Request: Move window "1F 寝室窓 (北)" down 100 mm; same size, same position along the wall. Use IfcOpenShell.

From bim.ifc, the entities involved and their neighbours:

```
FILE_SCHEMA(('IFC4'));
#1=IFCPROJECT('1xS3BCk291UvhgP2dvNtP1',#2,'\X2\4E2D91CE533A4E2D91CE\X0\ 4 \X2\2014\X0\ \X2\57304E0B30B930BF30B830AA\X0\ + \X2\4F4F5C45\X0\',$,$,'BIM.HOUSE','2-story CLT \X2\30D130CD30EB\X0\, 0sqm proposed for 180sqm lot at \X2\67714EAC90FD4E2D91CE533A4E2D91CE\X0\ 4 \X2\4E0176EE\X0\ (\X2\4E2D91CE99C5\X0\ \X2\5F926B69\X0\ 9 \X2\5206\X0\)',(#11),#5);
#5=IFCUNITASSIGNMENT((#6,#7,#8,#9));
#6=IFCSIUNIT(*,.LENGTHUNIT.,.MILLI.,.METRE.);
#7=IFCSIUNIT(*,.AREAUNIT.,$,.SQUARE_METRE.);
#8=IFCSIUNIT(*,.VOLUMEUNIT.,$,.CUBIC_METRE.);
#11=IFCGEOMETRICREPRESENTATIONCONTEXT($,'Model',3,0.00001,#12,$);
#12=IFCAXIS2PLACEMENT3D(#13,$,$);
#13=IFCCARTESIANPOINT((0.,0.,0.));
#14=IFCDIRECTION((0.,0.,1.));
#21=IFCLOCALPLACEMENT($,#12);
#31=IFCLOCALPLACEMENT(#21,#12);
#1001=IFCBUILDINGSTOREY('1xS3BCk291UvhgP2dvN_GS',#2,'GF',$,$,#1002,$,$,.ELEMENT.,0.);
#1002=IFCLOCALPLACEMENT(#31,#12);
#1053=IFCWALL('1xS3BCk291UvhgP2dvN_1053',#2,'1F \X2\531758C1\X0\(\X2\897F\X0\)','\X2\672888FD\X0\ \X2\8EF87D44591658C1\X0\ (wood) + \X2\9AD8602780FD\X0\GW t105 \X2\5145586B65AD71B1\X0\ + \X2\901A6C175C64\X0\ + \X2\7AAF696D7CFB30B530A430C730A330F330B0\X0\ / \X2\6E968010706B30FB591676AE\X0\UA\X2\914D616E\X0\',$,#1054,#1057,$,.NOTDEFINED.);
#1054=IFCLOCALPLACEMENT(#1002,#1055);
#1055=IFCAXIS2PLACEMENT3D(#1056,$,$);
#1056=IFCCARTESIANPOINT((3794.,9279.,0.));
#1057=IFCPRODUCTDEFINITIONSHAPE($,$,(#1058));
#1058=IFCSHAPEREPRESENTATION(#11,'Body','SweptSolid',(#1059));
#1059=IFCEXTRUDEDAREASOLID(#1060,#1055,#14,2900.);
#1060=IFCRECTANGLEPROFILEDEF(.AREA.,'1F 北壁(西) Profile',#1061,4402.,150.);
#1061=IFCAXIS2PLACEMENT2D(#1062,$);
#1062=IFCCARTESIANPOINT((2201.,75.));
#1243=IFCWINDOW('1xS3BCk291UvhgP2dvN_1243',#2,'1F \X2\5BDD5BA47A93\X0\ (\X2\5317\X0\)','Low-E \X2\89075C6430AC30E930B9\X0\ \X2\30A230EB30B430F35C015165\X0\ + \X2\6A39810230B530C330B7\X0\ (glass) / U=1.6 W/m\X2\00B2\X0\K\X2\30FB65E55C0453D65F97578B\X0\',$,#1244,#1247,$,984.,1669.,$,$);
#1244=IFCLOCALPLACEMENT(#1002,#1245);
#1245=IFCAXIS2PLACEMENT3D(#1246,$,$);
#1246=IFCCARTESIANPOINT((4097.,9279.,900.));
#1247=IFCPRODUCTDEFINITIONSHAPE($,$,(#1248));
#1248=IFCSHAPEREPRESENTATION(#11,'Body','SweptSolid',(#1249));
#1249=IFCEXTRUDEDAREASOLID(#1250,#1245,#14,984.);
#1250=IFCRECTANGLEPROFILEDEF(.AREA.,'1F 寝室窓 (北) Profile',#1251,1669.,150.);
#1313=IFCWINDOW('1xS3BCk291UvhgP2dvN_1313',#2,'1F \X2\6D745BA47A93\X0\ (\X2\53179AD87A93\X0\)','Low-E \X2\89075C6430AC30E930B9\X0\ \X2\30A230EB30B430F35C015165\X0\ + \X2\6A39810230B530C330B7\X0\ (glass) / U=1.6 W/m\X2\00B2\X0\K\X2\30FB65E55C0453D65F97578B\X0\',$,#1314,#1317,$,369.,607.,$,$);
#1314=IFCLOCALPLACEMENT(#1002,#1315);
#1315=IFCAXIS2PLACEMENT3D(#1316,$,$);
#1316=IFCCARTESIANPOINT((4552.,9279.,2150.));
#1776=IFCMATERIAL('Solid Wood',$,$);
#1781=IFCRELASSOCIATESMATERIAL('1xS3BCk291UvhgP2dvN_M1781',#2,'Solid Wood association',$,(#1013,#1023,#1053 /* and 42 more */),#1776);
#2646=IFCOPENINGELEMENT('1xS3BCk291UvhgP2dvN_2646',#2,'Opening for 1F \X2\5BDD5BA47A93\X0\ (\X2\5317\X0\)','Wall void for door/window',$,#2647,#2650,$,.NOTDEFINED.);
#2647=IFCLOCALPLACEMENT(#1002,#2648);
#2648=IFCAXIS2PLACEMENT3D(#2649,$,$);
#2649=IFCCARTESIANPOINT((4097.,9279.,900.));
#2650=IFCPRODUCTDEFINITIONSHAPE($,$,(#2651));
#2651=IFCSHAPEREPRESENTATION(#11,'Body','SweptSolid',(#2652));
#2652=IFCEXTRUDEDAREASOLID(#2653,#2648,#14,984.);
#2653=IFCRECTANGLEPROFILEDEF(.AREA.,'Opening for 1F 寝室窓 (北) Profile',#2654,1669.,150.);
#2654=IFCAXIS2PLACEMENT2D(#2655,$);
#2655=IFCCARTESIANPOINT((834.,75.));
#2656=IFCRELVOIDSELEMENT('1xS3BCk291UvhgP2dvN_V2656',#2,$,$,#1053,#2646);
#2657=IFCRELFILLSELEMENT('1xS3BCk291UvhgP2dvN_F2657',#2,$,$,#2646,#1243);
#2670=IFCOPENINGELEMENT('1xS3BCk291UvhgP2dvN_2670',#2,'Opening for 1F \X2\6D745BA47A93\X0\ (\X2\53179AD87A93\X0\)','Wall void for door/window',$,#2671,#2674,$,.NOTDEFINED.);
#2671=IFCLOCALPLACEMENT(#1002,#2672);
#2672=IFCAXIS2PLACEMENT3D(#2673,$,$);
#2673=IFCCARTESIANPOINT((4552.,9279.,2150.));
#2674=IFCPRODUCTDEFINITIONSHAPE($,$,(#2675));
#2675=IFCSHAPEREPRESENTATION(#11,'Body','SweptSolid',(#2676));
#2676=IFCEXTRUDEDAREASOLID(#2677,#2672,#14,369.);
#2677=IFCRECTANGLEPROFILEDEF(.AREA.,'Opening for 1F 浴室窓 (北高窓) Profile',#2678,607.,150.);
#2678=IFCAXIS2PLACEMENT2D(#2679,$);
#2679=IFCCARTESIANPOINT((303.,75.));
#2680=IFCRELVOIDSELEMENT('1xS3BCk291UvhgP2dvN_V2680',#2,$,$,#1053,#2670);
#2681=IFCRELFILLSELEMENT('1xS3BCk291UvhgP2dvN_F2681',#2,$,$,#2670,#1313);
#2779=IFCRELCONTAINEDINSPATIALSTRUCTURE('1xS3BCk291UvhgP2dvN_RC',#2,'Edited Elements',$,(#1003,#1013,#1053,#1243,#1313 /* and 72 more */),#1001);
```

```python
import numpy as np
import ifcopenshell
import ifcopenshell.api.geometry
import ifcopenshell.util.placement
import ifcopenshell.util.unit

model = ifcopenshell.open("bim.ifc")
unit_scale = ifcopenshell.util.unit.calculate_unit_scale(model)

window = model.by_id(1243)
opening = window.FillsVoids[0].RelatingOpeningElement
dz = -100.0

shift = np.array([0.0, 0.0, dz])
# The window is not placed relative to its opening, so move both.
for product in (opening, window):
    matrix = ifcopenshell.util.placement.get_local_placement(product.ObjectPlacement)
    matrix[:3, 3] += shift
    ifcopenshell.api.geometry.edit_object_placement(model, product=product, matrix=matrix, is_si=False)

print(f"moved by {dz * unit_scale:+.3f} m")

model.write("bim_updated.ifc")
```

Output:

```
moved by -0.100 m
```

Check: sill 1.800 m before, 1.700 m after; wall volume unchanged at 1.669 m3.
